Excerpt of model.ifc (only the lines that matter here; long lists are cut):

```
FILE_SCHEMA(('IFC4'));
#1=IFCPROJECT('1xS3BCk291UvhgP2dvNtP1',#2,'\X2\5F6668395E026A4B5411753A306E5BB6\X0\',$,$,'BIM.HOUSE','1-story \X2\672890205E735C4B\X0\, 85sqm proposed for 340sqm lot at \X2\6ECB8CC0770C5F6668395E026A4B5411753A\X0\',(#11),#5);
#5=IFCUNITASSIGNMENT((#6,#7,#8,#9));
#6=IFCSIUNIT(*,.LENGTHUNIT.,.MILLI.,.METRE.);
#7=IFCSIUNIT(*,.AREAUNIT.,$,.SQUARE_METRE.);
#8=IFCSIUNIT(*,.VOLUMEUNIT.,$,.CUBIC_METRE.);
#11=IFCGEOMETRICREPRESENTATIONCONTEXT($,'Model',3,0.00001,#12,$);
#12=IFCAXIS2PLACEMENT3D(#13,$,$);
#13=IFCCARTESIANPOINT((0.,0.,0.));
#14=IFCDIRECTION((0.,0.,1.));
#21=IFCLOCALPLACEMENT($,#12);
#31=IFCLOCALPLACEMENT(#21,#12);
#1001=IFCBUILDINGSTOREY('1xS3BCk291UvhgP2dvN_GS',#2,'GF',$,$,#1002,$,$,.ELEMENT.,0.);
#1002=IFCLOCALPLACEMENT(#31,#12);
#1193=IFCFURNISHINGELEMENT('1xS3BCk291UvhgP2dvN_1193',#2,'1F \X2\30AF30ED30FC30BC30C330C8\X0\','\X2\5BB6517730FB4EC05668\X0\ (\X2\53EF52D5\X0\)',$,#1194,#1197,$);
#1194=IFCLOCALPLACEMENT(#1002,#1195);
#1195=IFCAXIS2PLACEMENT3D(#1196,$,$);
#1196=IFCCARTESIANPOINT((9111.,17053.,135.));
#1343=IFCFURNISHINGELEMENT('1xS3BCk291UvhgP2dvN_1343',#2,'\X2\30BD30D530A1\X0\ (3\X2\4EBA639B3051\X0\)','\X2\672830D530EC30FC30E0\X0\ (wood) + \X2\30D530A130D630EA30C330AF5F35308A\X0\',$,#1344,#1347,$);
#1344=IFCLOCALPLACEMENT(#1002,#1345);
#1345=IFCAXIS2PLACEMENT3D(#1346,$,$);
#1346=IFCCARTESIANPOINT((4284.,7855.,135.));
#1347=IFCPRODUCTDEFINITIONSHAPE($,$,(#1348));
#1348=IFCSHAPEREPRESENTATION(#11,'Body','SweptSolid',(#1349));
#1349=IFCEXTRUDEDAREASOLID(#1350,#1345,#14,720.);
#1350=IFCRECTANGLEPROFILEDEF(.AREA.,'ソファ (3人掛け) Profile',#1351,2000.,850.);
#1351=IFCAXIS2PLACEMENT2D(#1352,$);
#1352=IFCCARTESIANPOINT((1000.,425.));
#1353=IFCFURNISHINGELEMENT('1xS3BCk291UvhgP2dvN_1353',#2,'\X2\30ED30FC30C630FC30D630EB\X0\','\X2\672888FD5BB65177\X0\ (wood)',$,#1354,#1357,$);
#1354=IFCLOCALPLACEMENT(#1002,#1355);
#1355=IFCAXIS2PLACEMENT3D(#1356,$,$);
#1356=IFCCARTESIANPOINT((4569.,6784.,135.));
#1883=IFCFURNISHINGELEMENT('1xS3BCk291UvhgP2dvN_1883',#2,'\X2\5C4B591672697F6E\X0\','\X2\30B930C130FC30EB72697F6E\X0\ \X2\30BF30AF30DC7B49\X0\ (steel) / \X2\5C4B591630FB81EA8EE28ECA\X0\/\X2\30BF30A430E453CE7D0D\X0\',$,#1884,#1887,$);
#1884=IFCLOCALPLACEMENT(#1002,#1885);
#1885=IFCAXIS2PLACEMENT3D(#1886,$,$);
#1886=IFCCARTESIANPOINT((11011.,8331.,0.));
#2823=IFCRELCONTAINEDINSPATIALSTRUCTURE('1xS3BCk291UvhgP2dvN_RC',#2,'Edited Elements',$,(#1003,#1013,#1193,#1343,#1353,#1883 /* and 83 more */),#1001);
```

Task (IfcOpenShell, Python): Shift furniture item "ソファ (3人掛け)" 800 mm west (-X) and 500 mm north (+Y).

```python
import ifcopenshell
import ifcopenshell.api.geometry
import ifcopenshell.util.placement
import ifcopenshell.util.unit

model = ifcopenshell.open("model.ifc")
unit_scale = ifcopenshell.util.unit.calculate_unit_scale(model)

item = model.by_guid("1xS3BCk291UvhgP2dvN_1343")
matrix = ifcopenshell.util.placement.get_local_placement(item.ObjectPlacement)
matrix[0, 3] -= 0.8 / unit_scale
matrix[1, 3] += 0.5 / unit_scale
ifcopenshell.api.geometry.edit_object_placement(model, product=item, matrix=matrix, is_si=False)

print(ifcopenshell.util.placement.get_local_placement(item.ObjectPlacement).round(3) + 0.0)

model.write("model_v2.ifc")
```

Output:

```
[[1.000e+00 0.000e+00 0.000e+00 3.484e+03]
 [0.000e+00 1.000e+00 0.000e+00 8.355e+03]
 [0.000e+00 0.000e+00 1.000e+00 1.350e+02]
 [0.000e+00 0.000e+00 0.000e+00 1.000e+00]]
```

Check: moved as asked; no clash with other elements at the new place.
